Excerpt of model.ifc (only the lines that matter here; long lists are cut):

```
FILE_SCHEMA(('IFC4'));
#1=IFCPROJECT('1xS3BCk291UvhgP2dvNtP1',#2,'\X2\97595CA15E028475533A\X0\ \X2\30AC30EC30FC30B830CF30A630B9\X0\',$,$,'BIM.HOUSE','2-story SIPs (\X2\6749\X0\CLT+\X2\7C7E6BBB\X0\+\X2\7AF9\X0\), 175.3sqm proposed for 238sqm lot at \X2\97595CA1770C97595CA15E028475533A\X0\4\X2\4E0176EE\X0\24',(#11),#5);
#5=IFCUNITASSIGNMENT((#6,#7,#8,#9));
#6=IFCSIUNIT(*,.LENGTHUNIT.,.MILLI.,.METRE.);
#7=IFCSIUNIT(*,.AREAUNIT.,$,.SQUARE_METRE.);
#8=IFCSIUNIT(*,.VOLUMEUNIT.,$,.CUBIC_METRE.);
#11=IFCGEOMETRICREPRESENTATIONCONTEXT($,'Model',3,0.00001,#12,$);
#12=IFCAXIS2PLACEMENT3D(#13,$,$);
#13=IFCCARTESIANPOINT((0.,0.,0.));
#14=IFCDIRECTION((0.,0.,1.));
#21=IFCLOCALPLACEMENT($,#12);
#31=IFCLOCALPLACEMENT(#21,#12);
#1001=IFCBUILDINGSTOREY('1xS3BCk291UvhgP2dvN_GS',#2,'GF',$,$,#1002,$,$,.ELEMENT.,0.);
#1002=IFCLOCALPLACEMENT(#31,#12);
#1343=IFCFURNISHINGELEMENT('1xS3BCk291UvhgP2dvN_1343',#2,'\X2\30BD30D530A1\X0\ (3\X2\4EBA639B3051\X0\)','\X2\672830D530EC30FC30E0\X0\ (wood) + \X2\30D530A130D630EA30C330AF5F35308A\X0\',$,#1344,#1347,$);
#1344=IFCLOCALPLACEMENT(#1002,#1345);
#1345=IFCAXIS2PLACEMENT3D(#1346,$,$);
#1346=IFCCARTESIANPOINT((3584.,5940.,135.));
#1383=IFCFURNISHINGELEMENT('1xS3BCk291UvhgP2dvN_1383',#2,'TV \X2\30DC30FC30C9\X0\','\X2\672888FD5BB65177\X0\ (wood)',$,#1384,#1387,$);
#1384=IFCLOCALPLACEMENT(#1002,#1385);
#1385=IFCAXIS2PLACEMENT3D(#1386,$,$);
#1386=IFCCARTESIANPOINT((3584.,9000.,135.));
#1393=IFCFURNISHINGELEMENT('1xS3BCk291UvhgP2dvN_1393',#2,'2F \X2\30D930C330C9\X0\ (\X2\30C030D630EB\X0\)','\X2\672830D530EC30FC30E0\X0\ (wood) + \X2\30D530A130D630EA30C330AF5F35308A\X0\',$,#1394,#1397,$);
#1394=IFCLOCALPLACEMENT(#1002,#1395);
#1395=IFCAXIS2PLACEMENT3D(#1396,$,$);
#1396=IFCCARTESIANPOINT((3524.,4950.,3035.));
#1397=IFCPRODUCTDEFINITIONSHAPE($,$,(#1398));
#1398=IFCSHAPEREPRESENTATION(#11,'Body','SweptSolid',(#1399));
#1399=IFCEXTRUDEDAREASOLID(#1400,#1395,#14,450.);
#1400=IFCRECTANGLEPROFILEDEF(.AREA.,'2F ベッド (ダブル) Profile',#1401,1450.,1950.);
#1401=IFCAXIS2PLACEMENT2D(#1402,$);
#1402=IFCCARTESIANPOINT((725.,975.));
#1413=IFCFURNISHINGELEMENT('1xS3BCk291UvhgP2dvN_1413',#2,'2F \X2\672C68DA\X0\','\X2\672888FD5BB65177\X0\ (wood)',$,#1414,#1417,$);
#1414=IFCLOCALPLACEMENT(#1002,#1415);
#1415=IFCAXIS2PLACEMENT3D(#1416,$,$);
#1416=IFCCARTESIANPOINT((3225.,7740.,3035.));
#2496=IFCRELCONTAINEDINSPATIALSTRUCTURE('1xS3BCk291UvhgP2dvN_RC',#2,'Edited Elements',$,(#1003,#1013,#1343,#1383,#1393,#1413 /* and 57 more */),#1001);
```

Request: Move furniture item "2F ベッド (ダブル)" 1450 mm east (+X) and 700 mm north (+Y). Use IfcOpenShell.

```python
import ifcopenshell
import ifcopenshell.api.geometry
import ifcopenshell.util.placement
import ifcopenshell.util.unit

model = ifcopenshell.open("model.ifc")
unit_scale = ifcopenshell.util.unit.calculate_unit_scale(model)

item = model.by_guid("1xS3BCk291UvhgP2dvN_1393")
matrix = ifcopenshell.util.placement.get_local_placement(item.ObjectPlacement)
matrix[0, 3] += 1.45 / unit_scale
matrix[1, 3] += 0.7 / unit_scale
ifcopenshell.api.geometry.edit_object_placement(model, product=item, matrix=matrix, is_si=False)

print(ifcopenshell.util.placement.get_local_placement(item.ObjectPlacement).round(3) + 0.0)

model.write("model_updated.ifc")
```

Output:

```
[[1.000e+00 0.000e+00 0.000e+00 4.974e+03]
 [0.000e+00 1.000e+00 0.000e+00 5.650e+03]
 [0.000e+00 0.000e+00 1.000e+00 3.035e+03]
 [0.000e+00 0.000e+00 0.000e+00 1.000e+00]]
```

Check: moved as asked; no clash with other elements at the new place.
